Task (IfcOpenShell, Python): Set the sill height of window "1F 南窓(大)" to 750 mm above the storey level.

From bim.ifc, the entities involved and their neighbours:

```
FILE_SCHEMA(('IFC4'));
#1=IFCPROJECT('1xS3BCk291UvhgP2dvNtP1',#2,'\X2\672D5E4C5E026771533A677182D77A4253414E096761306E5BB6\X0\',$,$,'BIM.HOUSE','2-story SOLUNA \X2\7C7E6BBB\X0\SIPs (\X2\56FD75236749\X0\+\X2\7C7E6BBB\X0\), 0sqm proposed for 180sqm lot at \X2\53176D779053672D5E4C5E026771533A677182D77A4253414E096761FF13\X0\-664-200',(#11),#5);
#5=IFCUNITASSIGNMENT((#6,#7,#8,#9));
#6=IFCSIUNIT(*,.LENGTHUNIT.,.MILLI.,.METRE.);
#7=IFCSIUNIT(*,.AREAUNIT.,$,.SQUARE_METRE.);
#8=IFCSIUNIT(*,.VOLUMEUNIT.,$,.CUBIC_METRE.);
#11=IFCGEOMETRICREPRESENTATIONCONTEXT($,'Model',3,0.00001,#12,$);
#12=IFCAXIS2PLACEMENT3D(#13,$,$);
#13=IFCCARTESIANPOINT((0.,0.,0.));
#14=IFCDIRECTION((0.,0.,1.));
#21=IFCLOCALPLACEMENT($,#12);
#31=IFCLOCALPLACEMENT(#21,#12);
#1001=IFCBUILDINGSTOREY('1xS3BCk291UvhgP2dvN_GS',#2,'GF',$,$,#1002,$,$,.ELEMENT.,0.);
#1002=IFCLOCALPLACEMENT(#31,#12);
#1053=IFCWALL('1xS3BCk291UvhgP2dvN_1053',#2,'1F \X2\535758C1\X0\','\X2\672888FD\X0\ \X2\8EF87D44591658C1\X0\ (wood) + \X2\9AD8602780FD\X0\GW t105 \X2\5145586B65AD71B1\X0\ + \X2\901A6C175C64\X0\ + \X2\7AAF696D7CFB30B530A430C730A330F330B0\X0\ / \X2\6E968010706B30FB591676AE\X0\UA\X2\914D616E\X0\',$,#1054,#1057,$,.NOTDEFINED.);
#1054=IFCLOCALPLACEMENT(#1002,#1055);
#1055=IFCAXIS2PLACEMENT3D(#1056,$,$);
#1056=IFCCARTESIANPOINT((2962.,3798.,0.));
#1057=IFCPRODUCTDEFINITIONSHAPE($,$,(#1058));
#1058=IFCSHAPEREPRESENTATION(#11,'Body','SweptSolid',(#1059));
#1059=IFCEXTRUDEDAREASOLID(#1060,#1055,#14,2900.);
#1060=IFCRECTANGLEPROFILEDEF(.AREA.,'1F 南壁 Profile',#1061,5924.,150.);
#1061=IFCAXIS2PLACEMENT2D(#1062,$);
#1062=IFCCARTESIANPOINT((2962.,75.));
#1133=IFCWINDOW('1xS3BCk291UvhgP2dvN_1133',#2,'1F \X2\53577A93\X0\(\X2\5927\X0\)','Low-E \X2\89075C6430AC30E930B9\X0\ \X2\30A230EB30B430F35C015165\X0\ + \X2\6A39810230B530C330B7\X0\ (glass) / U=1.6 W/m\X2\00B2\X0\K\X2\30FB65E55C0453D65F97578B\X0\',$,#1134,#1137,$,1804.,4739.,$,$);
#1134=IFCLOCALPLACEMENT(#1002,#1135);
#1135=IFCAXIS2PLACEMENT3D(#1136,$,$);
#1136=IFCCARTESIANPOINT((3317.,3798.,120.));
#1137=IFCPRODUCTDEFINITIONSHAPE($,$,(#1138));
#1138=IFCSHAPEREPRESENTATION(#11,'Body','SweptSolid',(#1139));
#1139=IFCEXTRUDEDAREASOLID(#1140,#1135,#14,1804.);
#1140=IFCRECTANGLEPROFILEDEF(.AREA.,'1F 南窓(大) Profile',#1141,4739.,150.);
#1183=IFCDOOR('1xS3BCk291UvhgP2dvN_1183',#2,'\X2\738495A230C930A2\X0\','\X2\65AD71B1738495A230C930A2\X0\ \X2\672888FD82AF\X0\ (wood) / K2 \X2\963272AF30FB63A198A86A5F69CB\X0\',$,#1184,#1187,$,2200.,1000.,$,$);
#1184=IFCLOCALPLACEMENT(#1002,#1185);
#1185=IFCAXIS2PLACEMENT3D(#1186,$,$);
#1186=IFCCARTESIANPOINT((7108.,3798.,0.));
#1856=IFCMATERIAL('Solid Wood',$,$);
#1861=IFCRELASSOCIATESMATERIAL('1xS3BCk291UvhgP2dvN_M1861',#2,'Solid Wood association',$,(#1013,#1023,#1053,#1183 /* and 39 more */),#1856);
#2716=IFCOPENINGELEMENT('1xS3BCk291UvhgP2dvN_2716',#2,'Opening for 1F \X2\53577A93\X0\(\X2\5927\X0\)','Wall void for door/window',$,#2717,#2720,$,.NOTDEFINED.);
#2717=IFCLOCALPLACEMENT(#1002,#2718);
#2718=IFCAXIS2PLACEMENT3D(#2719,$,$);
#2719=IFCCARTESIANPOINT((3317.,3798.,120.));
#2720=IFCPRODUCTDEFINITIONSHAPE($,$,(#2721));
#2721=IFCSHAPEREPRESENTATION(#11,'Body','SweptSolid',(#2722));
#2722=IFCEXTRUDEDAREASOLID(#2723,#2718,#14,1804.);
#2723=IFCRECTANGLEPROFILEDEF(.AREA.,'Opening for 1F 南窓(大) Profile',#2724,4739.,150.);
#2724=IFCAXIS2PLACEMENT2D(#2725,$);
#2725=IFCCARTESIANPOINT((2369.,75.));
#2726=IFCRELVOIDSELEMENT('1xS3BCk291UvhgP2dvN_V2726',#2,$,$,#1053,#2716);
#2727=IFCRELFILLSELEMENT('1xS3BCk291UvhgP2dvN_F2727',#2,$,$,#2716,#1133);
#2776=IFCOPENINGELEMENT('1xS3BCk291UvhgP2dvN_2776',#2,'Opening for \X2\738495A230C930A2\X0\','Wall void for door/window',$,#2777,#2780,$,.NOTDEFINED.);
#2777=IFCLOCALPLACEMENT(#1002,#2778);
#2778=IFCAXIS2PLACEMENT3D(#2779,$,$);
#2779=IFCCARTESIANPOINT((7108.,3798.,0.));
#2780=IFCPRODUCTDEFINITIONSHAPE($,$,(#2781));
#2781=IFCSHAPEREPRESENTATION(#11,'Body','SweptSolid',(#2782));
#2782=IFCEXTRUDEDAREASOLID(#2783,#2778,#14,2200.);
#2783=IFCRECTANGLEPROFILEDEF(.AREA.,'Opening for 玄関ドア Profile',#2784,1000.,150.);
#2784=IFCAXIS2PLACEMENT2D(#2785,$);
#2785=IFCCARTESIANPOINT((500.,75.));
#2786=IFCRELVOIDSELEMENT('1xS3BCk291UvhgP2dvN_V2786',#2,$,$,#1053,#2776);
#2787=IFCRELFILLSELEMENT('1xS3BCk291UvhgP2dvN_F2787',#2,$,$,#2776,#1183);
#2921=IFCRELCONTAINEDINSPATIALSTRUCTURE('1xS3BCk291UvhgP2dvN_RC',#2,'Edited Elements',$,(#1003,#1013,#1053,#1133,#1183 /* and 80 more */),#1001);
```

```python
import numpy as np
import ifcopenshell
import ifcopenshell.api.geometry
import ifcopenshell.geom
import ifcopenshell.util.element
import ifcopenshell.util.placement
import ifcopenshell.util.shape
import ifcopenshell.util.unit

model = ifcopenshell.open("bim.ifc")
unit_scale = ifcopenshell.util.unit.calculate_unit_scale(model)

window = model.by_guid("1xS3BCk291UvhgP2dvN_1133")
opening = window.FillsVoids[0].RelatingOpeningElement
storey = ifcopenshell.util.element.get_container(window, ifc_class="IfcBuildingStorey")
level = ifcopenshell.util.placement.get_local_placement(storey.ObjectPlacement)[2, 3]

# The opening's origin need not be at the sill, so measure its lowest point.
shape = ifcopenshell.geom.create_shape(ifcopenshell.geom.settings(), opening)
bottom = ifcopenshell.util.shape.get_shape_bottom_elevation(shape, shape.geometry) / unit_scale
dz = level + 0.75 / unit_scale - bottom

shift = np.array([0.0, 0.0, dz])
# The window is not placed relative to its opening, so move both.
for product in (opening, window):
    matrix = ifcopenshell.util.placement.get_local_placement(product.ObjectPlacement)
    matrix[:3, 3] += shift
    ifcopenshell.api.geometry.edit_object_placement(model, product=product, matrix=matrix, is_si=False)

print(f"moved by {dz * unit_scale:+.3f} m")

model.write("bim_updated.ifc")
```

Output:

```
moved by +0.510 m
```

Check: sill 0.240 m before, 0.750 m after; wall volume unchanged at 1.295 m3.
